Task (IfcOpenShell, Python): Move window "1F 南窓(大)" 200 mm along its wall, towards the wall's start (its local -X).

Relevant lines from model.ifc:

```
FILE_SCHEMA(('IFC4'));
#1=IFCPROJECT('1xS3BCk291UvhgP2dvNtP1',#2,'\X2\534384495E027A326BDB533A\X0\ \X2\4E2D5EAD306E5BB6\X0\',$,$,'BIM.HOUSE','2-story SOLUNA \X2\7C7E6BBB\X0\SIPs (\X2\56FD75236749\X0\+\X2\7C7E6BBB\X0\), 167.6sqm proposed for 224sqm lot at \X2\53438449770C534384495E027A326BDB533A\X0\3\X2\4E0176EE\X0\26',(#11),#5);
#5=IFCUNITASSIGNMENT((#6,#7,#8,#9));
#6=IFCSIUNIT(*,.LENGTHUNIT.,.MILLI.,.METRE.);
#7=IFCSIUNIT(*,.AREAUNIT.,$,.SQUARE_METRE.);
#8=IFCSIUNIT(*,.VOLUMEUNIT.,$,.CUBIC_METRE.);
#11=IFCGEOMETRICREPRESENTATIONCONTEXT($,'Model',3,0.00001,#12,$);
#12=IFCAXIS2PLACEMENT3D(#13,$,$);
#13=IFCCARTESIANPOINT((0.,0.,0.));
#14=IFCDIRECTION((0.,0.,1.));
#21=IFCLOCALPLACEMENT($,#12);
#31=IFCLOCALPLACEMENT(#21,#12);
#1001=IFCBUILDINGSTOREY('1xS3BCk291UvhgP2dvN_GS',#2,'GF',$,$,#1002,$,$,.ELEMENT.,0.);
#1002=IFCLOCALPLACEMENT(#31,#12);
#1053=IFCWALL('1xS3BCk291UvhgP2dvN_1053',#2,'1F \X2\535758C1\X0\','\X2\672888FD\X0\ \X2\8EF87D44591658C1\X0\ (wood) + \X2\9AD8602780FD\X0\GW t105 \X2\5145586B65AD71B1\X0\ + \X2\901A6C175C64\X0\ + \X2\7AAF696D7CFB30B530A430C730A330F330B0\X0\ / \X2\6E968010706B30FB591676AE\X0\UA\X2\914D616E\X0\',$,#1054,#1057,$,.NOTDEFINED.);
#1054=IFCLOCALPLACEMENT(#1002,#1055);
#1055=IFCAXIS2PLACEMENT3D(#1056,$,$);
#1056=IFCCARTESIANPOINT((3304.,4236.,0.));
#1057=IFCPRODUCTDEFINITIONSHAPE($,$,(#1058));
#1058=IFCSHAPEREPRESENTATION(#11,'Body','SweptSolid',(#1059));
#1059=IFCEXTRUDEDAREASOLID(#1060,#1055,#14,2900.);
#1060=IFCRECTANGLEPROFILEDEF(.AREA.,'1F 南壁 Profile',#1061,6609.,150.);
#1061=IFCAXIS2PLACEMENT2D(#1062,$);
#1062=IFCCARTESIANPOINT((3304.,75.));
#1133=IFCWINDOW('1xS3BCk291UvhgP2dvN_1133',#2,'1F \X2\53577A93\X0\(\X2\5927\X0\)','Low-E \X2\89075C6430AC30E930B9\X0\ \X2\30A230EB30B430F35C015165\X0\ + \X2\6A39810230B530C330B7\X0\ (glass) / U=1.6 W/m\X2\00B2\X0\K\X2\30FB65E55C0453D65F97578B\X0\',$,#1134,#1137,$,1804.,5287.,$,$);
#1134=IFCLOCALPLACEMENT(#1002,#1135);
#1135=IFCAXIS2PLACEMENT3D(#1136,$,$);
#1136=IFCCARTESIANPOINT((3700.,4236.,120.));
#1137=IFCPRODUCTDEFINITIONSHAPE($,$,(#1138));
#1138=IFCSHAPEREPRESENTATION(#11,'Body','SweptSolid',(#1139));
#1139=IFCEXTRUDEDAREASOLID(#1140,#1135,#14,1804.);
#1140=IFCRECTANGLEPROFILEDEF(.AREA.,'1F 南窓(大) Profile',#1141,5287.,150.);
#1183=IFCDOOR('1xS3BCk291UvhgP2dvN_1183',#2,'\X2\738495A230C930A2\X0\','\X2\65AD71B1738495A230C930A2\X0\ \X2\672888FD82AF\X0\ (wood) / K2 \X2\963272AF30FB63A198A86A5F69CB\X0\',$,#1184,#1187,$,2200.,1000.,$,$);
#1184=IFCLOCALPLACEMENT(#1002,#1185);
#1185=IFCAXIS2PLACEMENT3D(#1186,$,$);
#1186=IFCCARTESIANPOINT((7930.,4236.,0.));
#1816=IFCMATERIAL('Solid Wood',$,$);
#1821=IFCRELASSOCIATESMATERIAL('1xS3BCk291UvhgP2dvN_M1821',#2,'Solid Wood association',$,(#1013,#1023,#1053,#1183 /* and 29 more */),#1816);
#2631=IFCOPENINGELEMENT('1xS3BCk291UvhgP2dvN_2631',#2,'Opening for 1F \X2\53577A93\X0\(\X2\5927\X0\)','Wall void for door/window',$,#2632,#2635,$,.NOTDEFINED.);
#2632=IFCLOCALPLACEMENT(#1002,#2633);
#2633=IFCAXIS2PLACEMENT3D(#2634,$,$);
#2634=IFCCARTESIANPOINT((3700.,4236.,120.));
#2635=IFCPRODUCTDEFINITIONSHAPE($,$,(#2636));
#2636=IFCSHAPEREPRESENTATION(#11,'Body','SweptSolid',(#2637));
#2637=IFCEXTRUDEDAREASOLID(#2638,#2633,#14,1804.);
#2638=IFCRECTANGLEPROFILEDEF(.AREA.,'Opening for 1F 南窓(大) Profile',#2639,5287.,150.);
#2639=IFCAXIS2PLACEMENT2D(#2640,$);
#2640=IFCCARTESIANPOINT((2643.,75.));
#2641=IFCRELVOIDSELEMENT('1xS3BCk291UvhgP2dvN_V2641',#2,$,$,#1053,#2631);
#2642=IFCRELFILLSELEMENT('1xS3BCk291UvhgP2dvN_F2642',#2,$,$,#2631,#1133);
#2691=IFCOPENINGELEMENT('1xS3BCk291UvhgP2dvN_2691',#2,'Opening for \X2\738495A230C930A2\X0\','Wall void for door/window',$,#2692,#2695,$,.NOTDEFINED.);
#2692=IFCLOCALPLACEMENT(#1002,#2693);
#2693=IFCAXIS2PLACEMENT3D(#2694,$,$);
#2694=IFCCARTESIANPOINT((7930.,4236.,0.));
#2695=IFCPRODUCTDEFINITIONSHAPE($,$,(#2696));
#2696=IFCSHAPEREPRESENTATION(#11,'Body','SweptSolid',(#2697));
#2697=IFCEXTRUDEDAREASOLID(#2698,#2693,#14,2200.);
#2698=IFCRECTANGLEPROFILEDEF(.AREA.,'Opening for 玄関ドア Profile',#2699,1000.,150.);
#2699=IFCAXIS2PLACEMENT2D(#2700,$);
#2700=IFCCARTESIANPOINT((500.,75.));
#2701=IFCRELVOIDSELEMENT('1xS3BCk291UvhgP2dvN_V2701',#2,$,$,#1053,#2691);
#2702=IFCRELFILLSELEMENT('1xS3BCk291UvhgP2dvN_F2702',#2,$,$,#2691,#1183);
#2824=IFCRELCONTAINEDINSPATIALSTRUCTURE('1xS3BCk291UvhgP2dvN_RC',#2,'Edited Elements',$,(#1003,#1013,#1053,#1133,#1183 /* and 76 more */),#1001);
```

```python
import ifcopenshell
import ifcopenshell.api.geometry
import ifcopenshell.util.placement
import ifcopenshell.util.unit

model = ifcopenshell.open("model.ifc")
unit_scale = ifcopenshell.util.unit.calculate_unit_scale(model)

window = model.by_guid("1xS3BCk291UvhgP2dvN_1133")
opening = window.FillsVoids[0].RelatingOpeningElement
wall = opening.VoidsElements[0].RelatingBuildingElement

wall_matrix = ifcopenshell.util.placement.get_local_placement(wall.ObjectPlacement)
shift = wall_matrix[:3, 0] * -0.2 / unit_scale
before = ifcopenshell.util.placement.get_local_placement(window.ObjectPlacement)[:3, 3].copy()

# The window is not placed relative to its opening, so move both.
for product in (opening, window):
    matrix = ifcopenshell.util.placement.get_local_placement(product.ObjectPlacement)
    matrix[:3, 3] += shift
    ifcopenshell.api.geometry.edit_object_placement(model, product=product, matrix=matrix, is_si=False)

after = ifcopenshell.util.placement.get_local_placement(window.ObjectPlacement)[:3, 3]
print("window moved by", (after - before).round(3) + 0.0)

model.write("model_v2.ifc")
```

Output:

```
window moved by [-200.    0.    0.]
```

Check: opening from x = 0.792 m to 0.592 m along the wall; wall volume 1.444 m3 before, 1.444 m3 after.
